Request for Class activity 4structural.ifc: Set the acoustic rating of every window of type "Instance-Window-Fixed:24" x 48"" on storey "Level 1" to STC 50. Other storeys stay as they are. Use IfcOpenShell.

First a look at what the model holds.

```python
import ifcopenshell
import ifcopenshell.util.element

model = ifcopenshell.open("Class activity 4structural.ifc")
print(model.schema)
storey = next(s for s in model.by_type("IfcBuildingStorey") if s.Name == "Level 1")
windows = [e for e in ifcopenshell.util.element.get_decomposition(storey) if e.is_a("IfcWindow")]
seen = {}
for e in windows:
    element_type = ifcopenshell.util.element.get_type(e)
    key = (element_type.Name if element_type != e and element_type else None, ifcopenshell.util.element.get_pset(e, "Pset_WindowCommon", "AcousticRating"))
    seen[key] = seen.get(key, 0) + 1
for (name, value), count in sorted(seen.items(), key=str):
    print(count, "x", name, "|", value)
```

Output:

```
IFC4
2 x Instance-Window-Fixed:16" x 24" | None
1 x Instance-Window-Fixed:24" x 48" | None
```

```python
import ifcopenshell
import ifcopenshell.api.pset
import ifcopenshell.util.element

model = ifcopenshell.open("Class activity 4structural.ifc")

storey = next(s for s in model.by_type("IfcBuildingStorey") if s.Name == "Level 1")
windows = [e for e in ifcopenshell.util.element.get_decomposition(storey) if e.is_a("IfcWindow")]

count = 0
for e in windows:
    element_type = ifcopenshell.util.element.get_type(e)
    if element_type in (None, e) or element_type.Name != 'Instance-Window-Fixed:24" x 48"':
        continue
    # add_pset returns the element's existing set when there is one.
    pset = ifcopenshell.api.pset.add_pset(model, product=e, name="Pset_WindowCommon")
    ifcopenshell.api.pset.edit_pset(model, pset=pset, properties={"AcousticRating": "STC 50"})
    count += 1

print(count, "windows updated")

model.write("Class activity 4structural_v2.ifc")
```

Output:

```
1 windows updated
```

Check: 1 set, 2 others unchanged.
